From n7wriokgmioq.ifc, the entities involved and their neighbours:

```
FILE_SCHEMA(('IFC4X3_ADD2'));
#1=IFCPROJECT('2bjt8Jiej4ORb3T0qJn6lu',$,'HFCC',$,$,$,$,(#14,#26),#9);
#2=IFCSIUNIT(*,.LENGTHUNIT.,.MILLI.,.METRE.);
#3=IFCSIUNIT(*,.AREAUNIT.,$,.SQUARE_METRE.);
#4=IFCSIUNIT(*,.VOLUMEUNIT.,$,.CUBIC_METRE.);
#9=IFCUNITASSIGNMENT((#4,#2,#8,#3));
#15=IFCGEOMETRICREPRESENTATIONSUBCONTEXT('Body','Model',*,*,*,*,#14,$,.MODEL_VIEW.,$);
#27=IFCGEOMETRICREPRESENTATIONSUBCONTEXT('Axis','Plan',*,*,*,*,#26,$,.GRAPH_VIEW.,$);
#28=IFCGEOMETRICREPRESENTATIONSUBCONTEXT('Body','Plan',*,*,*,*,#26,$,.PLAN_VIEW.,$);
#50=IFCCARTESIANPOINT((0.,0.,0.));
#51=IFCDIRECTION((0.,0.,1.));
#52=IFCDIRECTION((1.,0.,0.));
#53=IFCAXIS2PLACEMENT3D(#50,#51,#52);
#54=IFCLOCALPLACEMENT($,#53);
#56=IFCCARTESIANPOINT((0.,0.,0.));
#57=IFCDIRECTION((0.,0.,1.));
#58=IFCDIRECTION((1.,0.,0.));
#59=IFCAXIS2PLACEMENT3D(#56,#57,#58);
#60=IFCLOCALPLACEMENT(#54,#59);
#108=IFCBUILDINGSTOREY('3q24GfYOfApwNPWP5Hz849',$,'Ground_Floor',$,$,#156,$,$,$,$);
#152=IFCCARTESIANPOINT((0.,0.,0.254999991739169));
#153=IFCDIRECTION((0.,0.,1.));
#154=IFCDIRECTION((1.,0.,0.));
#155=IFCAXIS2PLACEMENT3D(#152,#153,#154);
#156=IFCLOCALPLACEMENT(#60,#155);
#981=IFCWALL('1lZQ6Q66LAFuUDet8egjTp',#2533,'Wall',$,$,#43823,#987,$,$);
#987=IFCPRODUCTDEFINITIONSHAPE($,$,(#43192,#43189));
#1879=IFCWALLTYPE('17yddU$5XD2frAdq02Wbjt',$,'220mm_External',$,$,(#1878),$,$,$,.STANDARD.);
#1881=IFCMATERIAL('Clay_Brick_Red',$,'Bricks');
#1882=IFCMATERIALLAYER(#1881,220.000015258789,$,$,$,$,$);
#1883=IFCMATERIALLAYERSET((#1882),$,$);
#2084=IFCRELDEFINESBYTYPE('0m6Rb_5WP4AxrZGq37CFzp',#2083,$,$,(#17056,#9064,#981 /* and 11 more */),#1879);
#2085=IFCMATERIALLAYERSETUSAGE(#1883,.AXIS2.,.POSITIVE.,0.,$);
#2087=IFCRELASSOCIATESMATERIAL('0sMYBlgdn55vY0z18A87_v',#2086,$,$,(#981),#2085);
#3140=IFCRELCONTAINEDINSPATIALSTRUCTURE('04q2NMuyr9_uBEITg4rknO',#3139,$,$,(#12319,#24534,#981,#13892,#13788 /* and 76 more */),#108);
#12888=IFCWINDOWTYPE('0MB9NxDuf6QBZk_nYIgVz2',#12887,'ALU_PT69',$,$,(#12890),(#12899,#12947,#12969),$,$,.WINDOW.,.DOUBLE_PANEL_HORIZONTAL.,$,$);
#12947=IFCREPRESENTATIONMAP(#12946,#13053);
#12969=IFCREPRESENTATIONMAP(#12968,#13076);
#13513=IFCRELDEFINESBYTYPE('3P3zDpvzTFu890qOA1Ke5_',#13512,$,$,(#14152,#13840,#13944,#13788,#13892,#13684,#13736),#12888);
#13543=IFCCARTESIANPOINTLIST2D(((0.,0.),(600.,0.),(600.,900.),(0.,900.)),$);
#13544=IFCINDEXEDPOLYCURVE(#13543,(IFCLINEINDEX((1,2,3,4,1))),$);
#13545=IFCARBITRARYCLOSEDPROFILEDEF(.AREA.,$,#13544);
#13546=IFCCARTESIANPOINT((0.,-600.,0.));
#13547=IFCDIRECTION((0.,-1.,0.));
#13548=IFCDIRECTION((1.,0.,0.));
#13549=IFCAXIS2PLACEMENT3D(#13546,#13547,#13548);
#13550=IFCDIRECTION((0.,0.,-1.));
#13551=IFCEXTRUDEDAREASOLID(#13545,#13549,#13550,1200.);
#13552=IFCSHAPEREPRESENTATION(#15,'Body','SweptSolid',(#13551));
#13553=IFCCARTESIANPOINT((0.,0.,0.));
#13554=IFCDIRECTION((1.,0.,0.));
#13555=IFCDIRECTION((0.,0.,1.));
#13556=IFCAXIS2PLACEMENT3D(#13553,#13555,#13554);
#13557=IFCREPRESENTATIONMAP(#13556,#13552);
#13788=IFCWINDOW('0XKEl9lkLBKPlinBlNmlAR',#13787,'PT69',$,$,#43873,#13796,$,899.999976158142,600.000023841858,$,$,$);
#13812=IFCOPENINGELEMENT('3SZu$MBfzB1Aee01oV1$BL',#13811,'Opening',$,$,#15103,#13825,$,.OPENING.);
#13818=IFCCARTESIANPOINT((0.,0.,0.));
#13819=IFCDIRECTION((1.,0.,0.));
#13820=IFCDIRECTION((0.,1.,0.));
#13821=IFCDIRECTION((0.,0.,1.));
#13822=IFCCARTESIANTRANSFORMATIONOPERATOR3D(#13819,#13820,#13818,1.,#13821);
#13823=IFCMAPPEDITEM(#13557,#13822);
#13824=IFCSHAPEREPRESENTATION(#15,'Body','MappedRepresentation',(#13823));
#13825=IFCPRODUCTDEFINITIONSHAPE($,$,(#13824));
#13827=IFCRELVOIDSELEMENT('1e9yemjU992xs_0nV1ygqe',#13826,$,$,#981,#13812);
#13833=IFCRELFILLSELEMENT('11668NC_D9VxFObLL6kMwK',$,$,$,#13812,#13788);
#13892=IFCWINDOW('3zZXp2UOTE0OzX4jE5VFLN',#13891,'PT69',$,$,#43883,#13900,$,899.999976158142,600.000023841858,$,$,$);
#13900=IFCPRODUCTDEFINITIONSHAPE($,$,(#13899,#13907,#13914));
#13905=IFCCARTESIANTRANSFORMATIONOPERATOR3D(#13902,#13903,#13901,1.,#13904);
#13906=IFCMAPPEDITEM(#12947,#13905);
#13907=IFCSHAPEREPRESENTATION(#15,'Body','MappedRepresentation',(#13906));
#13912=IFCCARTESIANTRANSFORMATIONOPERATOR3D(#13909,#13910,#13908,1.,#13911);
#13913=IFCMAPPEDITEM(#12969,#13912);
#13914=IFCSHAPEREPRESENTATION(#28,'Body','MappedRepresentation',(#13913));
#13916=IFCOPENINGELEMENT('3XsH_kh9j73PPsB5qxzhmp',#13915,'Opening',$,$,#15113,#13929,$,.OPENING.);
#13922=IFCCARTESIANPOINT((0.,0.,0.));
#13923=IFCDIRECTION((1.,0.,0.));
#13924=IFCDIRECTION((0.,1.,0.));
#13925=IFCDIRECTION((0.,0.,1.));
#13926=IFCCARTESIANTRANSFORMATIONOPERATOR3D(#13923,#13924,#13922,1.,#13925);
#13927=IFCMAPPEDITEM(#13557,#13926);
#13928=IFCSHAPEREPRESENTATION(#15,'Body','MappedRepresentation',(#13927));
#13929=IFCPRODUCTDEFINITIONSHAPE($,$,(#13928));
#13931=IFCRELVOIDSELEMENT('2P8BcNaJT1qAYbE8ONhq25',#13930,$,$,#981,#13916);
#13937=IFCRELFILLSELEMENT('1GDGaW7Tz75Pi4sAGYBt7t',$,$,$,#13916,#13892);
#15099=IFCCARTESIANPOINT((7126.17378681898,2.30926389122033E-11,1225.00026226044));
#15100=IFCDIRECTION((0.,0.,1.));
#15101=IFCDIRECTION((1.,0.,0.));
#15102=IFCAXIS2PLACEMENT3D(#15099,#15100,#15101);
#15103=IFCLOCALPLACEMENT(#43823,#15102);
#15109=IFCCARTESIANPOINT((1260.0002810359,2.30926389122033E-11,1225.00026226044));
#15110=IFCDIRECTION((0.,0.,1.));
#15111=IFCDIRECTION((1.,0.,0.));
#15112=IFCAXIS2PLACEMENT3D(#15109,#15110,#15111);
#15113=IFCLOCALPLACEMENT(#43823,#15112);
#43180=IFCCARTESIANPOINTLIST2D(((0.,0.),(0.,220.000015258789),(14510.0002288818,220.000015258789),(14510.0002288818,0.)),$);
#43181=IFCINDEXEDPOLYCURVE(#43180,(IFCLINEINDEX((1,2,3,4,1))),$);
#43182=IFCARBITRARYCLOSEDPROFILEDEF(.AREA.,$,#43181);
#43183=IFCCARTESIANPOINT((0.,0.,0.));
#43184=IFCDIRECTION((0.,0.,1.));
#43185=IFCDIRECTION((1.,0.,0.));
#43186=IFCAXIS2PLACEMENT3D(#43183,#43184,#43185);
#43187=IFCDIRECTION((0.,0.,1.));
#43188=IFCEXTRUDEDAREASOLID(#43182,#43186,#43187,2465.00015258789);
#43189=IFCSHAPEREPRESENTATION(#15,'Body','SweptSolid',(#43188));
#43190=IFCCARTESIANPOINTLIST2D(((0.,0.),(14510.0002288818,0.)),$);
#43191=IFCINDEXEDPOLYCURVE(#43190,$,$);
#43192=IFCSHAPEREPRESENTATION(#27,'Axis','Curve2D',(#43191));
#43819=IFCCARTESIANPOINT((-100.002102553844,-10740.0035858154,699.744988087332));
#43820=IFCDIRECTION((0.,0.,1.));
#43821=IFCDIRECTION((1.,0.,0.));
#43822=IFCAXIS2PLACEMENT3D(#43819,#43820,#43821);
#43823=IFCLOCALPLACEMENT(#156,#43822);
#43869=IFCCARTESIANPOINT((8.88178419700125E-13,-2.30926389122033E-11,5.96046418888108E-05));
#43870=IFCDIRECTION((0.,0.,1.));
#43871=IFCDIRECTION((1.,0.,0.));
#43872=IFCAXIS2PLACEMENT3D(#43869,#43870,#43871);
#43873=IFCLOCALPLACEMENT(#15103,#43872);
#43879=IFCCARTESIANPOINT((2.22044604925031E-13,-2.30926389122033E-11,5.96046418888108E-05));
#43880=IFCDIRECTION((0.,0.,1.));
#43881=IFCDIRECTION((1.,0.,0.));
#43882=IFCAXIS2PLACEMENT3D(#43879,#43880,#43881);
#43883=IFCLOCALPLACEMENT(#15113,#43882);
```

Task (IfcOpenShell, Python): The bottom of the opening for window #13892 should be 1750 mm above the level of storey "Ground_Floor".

```python
import numpy as np
import ifcopenshell
import ifcopenshell.api.geometry
import ifcopenshell.geom
import ifcopenshell.util.element
import ifcopenshell.util.placement
import ifcopenshell.util.shape
import ifcopenshell.util.unit

model = ifcopenshell.open("n7wriokgmioq.ifc")
unit_scale = ifcopenshell.util.unit.calculate_unit_scale(model)

window = model.by_guid("3zZXp2UOTE0OzX4jE5VFLN")
opening = window.FillsVoids[0].RelatingOpeningElement
storey = ifcopenshell.util.element.get_container(window, ifc_class="IfcBuildingStorey")
level = ifcopenshell.util.placement.get_local_placement(storey.ObjectPlacement)[2, 3]

# The opening's origin need not be at the sill, so measure its lowest point.
shape = ifcopenshell.geom.create_shape(ifcopenshell.geom.settings(), opening)
bottom = ifcopenshell.util.shape.get_shape_bottom_elevation(shape, shape.geometry) / unit_scale
dz = level + 1.75 / unit_scale - bottom

shift = np.array([0.0, 0.0, dz])
# The window is placed relative to its opening, so it follows when the opening moves.
matrix = ifcopenshell.util.placement.get_local_placement(opening.ObjectPlacement)
matrix[:3, 3] += shift
ifcopenshell.api.geometry.edit_object_placement(
    model, product=opening, matrix=matrix, is_si=False, should_transform_children=True
)

print(f"moved by {dz * unit_scale:+.3f} m")

model.write("n7wriokgmioq_updated.ifc")
```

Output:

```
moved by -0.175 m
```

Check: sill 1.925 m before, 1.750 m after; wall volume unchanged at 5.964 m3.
